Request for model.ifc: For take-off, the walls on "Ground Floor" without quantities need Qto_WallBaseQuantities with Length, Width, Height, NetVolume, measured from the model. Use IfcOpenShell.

First a look at what the model holds.

```python
import ifcopenshell
import ifcopenshell.util.element
import ifcopenshell.util.unit

model = ifcopenshell.open("model.ifc")
print(model.schema)
for unit_type in ("LENGTHUNIT", "AREAUNIT", "VOLUMEUNIT"):
    print(unit_type, ifcopenshell.util.unit.calculate_unit_scale(model, unit_type))
storey = next(s for s in model.by_type("IfcBuildingStorey") if s.Name == "Ground Floor")
walls = [e for e in ifcopenshell.util.element.get_decomposition(storey) if e.is_a("IfcWall")]
for e in sorted(walls, key=lambda e: e.id()):
    print(e.id(), e.is_a(), e.Name, list(ifcopenshell.util.element.get_psets(e, qtos_only=True)), sep=" | ")
```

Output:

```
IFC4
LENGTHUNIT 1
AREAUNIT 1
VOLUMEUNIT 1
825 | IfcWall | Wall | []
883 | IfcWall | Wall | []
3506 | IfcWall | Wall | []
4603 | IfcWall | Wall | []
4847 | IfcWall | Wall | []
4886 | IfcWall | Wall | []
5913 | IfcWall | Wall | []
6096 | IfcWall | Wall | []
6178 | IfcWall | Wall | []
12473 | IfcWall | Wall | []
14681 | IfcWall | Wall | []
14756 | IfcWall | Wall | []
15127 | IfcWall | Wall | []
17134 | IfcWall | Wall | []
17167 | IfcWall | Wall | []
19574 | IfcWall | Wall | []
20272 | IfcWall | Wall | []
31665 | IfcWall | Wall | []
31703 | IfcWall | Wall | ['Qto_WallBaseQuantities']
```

```python
import ifcopenshell
import ifcopenshell.api.pset
import ifcopenshell.geom
import ifcopenshell.util.element
import ifcopenshell.util.shape
import ifcopenshell.util.unit

model = ifcopenshell.open("model.ifc")
unit_scale = ifcopenshell.util.unit.calculate_unit_scale(model)
volume_scale = ifcopenshell.util.unit.calculate_unit_scale(model, "VOLUMEUNIT")
settings = ifcopenshell.geom.settings()

storey = next(s for s in model.by_type("IfcBuildingStorey") if s.Name == "Ground Floor")
walls = [e for e in ifcopenshell.util.element.get_decomposition(storey) if e.is_a("IfcWall")]

for e in sorted(walls, key=lambda e: e.id()):
    if ifcopenshell.util.element.get_psets(e, qtos_only=True, should_inherit=False):
        continue
    # Geometry comes back in metres, in the element's own axes.
    shape = ifcopenshell.geom.create_shape(settings, e)
    values = {
        "Length": ifcopenshell.util.shape.get_x(shape.geometry) / unit_scale,
        "Width": ifcopenshell.util.shape.get_y(shape.geometry) / unit_scale,
        "Height": ifcopenshell.util.shape.get_z(shape.geometry) / unit_scale,
        "NetVolume": ifcopenshell.util.shape.get_volume(shape.geometry) / volume_scale,
    }
    qto = ifcopenshell.api.pset.add_qto(model, product=e, name="Qto_WallBaseQuantities")
    ifcopenshell.api.pset.edit_qto(model, qto=qto, properties=values)
    print(e.id(), {k: round(v, 3) for k, v in values.items()})

model.write("model_rev.ifc")
```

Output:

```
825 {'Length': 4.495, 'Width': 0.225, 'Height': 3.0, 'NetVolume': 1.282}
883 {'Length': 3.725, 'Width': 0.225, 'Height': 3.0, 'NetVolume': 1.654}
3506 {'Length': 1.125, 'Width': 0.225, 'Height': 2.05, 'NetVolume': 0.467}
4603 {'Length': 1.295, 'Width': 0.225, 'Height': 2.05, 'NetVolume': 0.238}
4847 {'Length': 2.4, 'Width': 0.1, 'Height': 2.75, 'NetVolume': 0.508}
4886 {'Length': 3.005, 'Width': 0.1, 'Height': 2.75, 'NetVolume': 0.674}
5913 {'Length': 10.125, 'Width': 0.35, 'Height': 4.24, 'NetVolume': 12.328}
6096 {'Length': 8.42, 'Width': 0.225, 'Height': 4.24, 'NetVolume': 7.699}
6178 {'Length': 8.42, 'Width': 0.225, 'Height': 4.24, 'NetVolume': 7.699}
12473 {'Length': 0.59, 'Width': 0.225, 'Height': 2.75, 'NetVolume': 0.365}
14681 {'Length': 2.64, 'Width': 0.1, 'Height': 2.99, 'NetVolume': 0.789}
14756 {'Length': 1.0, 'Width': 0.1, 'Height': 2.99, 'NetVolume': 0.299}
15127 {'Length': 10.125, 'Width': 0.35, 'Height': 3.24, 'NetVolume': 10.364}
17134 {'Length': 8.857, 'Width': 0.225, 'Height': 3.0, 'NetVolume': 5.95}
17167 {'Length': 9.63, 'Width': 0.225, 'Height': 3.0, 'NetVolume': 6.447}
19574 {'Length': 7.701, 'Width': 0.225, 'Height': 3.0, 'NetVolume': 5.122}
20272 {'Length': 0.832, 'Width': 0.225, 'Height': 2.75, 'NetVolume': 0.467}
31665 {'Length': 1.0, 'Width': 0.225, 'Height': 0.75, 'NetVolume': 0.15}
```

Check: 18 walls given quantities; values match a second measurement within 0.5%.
